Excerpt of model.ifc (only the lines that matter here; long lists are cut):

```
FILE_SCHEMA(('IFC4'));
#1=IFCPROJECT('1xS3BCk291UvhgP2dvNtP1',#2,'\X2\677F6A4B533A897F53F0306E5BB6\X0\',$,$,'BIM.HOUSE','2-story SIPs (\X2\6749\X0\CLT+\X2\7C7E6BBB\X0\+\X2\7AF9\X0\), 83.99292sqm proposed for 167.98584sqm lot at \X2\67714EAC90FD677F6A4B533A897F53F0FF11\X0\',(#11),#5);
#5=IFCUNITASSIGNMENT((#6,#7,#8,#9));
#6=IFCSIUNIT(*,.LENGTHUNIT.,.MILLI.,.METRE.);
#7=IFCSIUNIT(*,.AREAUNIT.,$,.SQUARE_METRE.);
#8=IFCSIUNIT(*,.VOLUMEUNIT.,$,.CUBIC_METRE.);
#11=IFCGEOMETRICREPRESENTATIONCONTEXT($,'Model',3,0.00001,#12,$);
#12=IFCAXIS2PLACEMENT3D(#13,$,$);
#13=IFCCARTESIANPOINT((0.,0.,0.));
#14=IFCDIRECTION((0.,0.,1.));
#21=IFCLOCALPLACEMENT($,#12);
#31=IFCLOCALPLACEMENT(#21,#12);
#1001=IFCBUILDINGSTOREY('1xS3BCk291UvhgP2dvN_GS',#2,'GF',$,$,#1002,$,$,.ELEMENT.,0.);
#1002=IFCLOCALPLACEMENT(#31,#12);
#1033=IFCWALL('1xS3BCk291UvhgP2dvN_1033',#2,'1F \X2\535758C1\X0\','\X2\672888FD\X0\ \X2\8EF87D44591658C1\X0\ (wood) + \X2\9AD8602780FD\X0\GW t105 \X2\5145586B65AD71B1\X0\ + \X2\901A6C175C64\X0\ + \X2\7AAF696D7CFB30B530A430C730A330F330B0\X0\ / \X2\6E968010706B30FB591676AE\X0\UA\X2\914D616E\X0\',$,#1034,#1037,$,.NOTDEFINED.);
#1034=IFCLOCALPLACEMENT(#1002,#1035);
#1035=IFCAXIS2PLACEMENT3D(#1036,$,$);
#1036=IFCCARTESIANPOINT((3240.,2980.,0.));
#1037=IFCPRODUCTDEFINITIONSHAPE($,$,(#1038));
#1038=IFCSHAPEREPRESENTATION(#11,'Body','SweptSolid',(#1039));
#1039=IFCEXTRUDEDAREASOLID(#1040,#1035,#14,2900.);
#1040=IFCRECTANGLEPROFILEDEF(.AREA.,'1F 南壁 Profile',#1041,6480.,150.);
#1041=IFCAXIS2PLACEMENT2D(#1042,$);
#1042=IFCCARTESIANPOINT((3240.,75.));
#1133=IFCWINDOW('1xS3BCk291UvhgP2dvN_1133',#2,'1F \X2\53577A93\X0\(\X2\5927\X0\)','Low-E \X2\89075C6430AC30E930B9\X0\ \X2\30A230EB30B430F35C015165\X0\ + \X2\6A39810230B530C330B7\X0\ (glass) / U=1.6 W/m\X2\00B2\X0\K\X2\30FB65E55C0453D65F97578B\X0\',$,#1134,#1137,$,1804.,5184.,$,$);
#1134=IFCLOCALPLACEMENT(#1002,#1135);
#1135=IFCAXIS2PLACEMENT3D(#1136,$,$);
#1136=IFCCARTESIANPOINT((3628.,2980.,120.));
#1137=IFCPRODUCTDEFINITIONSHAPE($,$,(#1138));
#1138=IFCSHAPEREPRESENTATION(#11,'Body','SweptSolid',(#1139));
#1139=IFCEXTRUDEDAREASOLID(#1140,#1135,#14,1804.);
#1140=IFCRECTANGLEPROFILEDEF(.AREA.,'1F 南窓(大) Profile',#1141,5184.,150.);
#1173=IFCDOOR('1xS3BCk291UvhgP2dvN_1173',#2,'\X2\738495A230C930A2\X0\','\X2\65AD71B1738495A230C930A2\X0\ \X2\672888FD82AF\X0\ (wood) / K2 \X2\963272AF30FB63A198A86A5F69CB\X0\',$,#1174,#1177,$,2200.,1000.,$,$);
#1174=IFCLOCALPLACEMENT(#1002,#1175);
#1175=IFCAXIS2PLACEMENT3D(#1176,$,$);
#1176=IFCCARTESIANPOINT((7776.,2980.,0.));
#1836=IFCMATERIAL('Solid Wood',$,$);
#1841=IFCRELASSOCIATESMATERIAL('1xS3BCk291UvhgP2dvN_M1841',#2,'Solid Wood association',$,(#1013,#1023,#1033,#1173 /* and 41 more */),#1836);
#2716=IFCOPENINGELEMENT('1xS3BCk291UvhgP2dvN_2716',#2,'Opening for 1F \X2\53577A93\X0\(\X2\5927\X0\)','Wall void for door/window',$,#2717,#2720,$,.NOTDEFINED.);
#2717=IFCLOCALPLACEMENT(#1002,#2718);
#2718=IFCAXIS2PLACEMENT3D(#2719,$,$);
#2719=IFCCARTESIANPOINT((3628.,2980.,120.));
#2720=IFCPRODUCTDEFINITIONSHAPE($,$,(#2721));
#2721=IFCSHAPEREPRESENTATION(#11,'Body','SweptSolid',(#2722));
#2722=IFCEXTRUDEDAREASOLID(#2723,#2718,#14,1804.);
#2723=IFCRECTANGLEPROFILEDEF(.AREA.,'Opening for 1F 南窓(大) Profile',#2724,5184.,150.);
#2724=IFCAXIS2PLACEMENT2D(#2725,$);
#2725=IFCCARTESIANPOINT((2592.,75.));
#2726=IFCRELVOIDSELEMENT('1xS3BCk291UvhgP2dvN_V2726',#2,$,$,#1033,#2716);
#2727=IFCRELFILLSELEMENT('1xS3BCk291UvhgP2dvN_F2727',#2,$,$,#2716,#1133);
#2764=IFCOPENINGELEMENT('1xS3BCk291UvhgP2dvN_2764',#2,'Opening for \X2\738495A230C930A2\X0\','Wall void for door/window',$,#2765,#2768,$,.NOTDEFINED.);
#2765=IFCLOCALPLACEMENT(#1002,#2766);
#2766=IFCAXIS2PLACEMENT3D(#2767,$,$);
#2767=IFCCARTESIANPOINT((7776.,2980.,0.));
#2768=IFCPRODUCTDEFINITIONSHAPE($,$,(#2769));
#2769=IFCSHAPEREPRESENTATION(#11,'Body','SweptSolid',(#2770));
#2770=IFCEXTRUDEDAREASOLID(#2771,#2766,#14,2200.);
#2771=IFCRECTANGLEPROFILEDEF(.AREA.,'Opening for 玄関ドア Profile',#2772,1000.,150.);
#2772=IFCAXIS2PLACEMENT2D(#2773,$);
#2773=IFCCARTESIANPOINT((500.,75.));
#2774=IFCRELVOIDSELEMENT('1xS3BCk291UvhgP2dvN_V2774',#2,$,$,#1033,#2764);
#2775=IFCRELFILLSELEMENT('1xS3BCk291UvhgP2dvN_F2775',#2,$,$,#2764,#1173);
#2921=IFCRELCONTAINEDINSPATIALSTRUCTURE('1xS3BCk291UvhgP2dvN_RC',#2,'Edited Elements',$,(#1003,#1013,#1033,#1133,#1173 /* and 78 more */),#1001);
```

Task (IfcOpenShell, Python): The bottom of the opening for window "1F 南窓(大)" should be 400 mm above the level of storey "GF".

```python
import numpy as np
import ifcopenshell
import ifcopenshell.api.geometry
import ifcopenshell.geom
import ifcopenshell.util.element
import ifcopenshell.util.placement
import ifcopenshell.util.shape
import ifcopenshell.util.unit

model = ifcopenshell.open("model.ifc")
unit_scale = ifcopenshell.util.unit.calculate_unit_scale(model)

window = model.by_guid("1xS3BCk291UvhgP2dvN_1133")
opening = window.FillsVoids[0].RelatingOpeningElement
storey = ifcopenshell.util.element.get_container(window, ifc_class="IfcBuildingStorey")
level = ifcopenshell.util.placement.get_local_placement(storey.ObjectPlacement)[2, 3]

# The opening's origin need not be at the sill, so measure its lowest point.
shape = ifcopenshell.geom.create_shape(ifcopenshell.geom.settings(), opening)
bottom = ifcopenshell.util.shape.get_shape_bottom_elevation(shape, shape.geometry) / unit_scale
dz = level + 400.0 - bottom

shift = np.array([0.0, 0.0, dz])
# The window is not placed relative to its opening, so move both.
for product in (opening, window):
    matrix = ifcopenshell.util.placement.get_local_placement(product.ObjectPlacement)
    matrix[:3, 3] += shift
    ifcopenshell.api.geometry.edit_object_placement(model, product=product, matrix=matrix, is_si=False)

print(f"moved by {dz * unit_scale:+.3f} m")

model.write("model_v2.ifc")
```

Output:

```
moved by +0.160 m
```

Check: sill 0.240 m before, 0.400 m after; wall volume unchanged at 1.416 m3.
